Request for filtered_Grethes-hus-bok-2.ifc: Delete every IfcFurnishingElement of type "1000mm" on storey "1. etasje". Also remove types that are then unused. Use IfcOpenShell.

First a look at what the model holds.

```python
import ifcopenshell
import ifcopenshell.util.element

model = ifcopenshell.open("filtered_Grethes-hus-bok-2.ifc")
print(model.schema)
storey = next(s for s in model.by_type("IfcBuildingStorey") if s.Name == "1. etasje")
furniture = [e for e in ifcopenshell.util.element.get_decomposition(storey) if e.is_a("IfcFurnishingElement")]
seen = {}
for e in furniture:
    element_type = ifcopenshell.util.element.get_type(e)
    name = element_type.Name if element_type not in (None, e) else None
    seen[name] = seen.get(name, 0) + 1
for name, count in sorted(seen.items(), key=str):
    print(count, "x", name)
```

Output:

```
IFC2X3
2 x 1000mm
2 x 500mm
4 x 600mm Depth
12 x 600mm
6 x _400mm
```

```python
import ifcopenshell
import ifcopenshell.api.root
import ifcopenshell.util.element

model = ifcopenshell.open("filtered_Grethes-hus-bok-2.ifc")

storey = next(s for s in model.by_type("IfcBuildingStorey") if s.Name == "1. etasje")
furniture = [e for e in ifcopenshell.util.element.get_decomposition(storey) if e.is_a("IfcFurnishingElement")]
targets = [e for e in furniture if (t := ifcopenshell.util.element.get_type(e)) not in (None, e) and t.Name == "1000mm"]
types = {ifcopenshell.util.element.get_type(e) for e in targets} - {None, *targets}

for e in targets:
    ifcopenshell.api.root.remove_product(model, product=e)
print(len(targets), "removed")

unused = [t for t in types if not ifcopenshell.util.element.get_types(t)]
for t in unused:
    ifcopenshell.api.root.remove_product(model, product=t)
print(len(unused), "unused types removed")

model.write("filtered_Grethes-hus-bok-2_rev.ifc")
```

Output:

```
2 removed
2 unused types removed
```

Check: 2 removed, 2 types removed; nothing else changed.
